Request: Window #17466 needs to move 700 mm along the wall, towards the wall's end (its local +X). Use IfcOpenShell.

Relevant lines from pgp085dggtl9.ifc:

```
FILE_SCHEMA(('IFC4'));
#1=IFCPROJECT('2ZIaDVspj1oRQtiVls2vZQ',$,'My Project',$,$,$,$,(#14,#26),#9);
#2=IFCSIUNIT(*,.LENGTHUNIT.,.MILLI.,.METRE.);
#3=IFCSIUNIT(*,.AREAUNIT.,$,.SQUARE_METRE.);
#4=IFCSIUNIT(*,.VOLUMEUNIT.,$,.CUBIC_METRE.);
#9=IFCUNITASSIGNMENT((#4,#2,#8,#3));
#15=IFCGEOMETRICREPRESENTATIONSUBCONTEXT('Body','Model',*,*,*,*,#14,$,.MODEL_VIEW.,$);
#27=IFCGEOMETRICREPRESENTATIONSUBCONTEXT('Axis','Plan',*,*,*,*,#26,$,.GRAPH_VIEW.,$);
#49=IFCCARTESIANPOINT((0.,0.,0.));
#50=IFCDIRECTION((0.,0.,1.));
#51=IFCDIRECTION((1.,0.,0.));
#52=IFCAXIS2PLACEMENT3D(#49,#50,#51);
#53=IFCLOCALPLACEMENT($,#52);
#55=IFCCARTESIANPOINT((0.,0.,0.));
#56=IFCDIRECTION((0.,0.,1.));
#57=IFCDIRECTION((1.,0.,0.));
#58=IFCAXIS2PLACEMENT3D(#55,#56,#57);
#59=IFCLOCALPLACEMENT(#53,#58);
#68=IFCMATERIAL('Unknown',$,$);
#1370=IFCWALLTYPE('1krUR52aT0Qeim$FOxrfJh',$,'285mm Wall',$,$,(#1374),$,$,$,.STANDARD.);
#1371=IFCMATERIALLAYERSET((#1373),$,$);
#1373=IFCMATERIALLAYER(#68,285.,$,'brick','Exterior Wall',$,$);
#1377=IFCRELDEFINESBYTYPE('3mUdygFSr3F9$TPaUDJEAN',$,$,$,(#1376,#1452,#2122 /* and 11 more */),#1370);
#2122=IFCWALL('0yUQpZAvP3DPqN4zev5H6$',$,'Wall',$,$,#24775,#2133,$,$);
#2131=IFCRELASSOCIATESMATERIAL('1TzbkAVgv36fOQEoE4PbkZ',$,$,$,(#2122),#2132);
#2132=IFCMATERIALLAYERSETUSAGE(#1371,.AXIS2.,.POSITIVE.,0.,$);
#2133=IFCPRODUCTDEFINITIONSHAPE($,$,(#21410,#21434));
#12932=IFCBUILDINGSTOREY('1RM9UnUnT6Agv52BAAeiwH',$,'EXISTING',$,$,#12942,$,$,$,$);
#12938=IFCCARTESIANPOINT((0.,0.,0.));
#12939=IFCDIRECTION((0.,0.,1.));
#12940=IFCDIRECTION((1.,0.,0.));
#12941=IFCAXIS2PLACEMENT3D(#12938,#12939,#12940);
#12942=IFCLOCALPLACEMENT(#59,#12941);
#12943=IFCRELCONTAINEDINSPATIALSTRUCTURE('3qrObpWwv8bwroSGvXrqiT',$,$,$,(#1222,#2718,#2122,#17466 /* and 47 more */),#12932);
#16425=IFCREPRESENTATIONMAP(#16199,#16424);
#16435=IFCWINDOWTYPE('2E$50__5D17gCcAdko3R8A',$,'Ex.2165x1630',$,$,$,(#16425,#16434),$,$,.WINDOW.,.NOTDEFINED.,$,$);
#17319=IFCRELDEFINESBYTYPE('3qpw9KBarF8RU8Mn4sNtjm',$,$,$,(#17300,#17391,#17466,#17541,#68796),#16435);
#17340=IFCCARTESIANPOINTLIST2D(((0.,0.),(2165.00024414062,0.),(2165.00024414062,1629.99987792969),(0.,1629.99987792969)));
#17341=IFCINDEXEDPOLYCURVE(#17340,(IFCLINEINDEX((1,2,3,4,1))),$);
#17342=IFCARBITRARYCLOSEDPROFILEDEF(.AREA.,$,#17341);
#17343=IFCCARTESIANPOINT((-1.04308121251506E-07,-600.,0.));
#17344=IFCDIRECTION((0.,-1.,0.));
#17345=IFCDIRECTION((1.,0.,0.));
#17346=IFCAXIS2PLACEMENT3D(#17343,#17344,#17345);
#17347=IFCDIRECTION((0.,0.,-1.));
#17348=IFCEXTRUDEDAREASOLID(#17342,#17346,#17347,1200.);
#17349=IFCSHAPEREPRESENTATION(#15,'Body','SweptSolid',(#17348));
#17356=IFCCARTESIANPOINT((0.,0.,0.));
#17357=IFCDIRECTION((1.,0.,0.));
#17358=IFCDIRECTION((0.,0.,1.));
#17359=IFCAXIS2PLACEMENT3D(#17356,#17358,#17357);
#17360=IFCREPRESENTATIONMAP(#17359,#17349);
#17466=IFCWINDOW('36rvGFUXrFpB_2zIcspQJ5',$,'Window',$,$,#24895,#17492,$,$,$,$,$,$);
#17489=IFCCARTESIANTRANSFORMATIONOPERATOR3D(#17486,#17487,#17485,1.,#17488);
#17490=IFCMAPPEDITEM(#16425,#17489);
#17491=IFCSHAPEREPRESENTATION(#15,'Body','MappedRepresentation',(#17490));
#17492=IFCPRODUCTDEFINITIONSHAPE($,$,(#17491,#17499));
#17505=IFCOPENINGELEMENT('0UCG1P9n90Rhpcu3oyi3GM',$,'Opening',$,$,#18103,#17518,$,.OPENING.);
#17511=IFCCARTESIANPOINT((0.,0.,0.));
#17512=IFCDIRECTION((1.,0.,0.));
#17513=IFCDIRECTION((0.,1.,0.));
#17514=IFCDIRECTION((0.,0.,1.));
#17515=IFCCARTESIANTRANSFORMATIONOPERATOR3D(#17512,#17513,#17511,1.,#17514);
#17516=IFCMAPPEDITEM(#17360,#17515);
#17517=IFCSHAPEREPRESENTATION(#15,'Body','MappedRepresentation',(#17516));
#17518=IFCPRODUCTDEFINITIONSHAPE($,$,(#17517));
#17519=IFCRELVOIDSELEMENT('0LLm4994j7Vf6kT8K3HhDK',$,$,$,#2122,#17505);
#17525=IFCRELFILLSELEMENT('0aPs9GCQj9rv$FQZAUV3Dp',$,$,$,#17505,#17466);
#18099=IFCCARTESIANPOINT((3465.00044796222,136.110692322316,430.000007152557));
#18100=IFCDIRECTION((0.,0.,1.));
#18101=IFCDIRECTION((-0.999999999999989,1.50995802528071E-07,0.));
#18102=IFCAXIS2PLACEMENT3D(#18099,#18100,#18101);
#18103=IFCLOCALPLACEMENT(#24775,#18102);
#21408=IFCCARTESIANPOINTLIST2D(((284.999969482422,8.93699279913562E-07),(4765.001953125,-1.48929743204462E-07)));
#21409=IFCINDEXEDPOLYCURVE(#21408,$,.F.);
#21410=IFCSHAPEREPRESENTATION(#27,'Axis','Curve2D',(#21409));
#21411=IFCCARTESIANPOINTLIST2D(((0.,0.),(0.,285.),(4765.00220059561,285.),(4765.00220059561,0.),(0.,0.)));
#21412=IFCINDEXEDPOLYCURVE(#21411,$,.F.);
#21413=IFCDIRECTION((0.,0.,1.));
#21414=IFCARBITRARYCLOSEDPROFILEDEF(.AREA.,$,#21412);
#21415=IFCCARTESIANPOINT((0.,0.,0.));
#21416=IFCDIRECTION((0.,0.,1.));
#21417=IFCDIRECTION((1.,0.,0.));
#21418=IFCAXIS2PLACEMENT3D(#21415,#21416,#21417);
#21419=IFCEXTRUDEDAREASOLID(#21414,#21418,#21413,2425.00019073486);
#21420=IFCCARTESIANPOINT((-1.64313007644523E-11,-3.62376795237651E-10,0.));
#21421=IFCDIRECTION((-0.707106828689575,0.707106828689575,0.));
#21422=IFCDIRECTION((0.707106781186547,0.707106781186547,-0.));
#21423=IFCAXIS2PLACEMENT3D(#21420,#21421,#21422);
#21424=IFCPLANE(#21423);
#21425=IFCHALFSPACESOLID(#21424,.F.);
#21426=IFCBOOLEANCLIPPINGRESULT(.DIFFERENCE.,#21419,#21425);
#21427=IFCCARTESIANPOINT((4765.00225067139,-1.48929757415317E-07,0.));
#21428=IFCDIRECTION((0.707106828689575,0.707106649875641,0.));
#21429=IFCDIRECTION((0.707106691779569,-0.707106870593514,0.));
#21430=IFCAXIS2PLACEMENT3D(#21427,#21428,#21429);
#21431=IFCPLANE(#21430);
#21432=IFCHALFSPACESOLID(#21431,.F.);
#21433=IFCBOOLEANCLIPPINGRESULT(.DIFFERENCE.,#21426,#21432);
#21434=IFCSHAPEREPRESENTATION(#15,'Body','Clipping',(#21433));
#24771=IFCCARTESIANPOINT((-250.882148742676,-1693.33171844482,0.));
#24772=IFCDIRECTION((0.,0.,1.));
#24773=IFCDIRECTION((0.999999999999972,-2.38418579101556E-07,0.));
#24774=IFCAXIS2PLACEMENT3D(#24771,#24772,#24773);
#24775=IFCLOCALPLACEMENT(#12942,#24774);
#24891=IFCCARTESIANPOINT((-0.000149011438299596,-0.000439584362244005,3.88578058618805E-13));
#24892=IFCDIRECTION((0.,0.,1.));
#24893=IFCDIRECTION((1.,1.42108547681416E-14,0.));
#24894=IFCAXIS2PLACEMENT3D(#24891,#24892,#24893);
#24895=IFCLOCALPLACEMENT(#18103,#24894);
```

```python
import ifcopenshell
import ifcopenshell.api.geometry
import ifcopenshell.util.placement
import ifcopenshell.util.unit

model = ifcopenshell.open("pgp085dggtl9.ifc")
unit_scale = ifcopenshell.util.unit.calculate_unit_scale(model)

window = model.by_id(17466)
opening = window.FillsVoids[0].RelatingOpeningElement
wall = opening.VoidsElements[0].RelatingBuildingElement

wall_matrix = ifcopenshell.util.placement.get_local_placement(wall.ObjectPlacement)
shift = wall_matrix[:3, 0] * 0.7 / unit_scale
before = ifcopenshell.util.placement.get_local_placement(window.ObjectPlacement)[:3, 3].copy()

# The window is placed relative to its opening, so it follows when the opening moves.
matrix = ifcopenshell.util.placement.get_local_placement(opening.ObjectPlacement)
matrix[:3, 3] += shift
ifcopenshell.api.geometry.edit_object_placement(
    model, product=opening, matrix=matrix, is_si=False, should_transform_children=True
)

after = ifcopenshell.util.placement.get_local_placement(window.ObjectPlacement)[:3, 3]
print("window moved by", (after - before).round(3) + 0.0)

model.write("pgp085dggtl9_rev.ifc")
```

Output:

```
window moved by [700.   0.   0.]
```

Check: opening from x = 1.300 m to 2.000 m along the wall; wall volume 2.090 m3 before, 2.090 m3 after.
